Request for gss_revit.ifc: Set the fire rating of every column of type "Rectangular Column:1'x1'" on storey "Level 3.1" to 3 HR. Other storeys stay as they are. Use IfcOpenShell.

First a look at what the model holds.

```python
import ifcopenshell
import ifcopenshell.util.element

model = ifcopenshell.open("gss_revit.ifc")
print(model.schema)
storey = next(s for s in model.by_type("IfcBuildingStorey") if s.Name == "Level 3.1")
columns = [e for e in ifcopenshell.util.element.get_decomposition(storey) if e.is_a("IfcColumn")]
seen = {}
for e in columns:
    element_type = ifcopenshell.util.element.get_type(e)
    key = (element_type.Name if element_type != e and element_type else None, ifcopenshell.util.element.get_pset(e, "Pset_ColumnCommon", "FireRating"))
    seen[key] = seen.get(key, 0) + 1
for (name, value), count in sorted(seen.items(), key=str):
    print(count, "x", name, "|", value)
```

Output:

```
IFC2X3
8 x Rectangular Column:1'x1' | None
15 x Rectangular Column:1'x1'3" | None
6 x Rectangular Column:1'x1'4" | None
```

```python
import ifcopenshell
import ifcopenshell.api.pset
import ifcopenshell.util.element

model = ifcopenshell.open("gss_revit.ifc")

storey = next(s for s in model.by_type("IfcBuildingStorey") if s.Name == "Level 3.1")
columns = [e for e in ifcopenshell.util.element.get_decomposition(storey) if e.is_a("IfcColumn")]

count = 0
for e in columns:
    element_type = ifcopenshell.util.element.get_type(e)
    if element_type in (None, e) or element_type.Name != "Rectangular Column:1'x1'":
        continue
    # add_pset returns the element's existing set when there is one.
    pset = ifcopenshell.api.pset.add_pset(model, product=e, name="Pset_ColumnCommon")
    ifcopenshell.api.pset.edit_pset(model, pset=pset, properties={"FireRating": "3 HR"})
    count += 1

print(count, "columns updated")

model.write("gss_revit_updated.ifc")
```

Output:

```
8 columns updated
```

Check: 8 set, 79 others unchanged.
